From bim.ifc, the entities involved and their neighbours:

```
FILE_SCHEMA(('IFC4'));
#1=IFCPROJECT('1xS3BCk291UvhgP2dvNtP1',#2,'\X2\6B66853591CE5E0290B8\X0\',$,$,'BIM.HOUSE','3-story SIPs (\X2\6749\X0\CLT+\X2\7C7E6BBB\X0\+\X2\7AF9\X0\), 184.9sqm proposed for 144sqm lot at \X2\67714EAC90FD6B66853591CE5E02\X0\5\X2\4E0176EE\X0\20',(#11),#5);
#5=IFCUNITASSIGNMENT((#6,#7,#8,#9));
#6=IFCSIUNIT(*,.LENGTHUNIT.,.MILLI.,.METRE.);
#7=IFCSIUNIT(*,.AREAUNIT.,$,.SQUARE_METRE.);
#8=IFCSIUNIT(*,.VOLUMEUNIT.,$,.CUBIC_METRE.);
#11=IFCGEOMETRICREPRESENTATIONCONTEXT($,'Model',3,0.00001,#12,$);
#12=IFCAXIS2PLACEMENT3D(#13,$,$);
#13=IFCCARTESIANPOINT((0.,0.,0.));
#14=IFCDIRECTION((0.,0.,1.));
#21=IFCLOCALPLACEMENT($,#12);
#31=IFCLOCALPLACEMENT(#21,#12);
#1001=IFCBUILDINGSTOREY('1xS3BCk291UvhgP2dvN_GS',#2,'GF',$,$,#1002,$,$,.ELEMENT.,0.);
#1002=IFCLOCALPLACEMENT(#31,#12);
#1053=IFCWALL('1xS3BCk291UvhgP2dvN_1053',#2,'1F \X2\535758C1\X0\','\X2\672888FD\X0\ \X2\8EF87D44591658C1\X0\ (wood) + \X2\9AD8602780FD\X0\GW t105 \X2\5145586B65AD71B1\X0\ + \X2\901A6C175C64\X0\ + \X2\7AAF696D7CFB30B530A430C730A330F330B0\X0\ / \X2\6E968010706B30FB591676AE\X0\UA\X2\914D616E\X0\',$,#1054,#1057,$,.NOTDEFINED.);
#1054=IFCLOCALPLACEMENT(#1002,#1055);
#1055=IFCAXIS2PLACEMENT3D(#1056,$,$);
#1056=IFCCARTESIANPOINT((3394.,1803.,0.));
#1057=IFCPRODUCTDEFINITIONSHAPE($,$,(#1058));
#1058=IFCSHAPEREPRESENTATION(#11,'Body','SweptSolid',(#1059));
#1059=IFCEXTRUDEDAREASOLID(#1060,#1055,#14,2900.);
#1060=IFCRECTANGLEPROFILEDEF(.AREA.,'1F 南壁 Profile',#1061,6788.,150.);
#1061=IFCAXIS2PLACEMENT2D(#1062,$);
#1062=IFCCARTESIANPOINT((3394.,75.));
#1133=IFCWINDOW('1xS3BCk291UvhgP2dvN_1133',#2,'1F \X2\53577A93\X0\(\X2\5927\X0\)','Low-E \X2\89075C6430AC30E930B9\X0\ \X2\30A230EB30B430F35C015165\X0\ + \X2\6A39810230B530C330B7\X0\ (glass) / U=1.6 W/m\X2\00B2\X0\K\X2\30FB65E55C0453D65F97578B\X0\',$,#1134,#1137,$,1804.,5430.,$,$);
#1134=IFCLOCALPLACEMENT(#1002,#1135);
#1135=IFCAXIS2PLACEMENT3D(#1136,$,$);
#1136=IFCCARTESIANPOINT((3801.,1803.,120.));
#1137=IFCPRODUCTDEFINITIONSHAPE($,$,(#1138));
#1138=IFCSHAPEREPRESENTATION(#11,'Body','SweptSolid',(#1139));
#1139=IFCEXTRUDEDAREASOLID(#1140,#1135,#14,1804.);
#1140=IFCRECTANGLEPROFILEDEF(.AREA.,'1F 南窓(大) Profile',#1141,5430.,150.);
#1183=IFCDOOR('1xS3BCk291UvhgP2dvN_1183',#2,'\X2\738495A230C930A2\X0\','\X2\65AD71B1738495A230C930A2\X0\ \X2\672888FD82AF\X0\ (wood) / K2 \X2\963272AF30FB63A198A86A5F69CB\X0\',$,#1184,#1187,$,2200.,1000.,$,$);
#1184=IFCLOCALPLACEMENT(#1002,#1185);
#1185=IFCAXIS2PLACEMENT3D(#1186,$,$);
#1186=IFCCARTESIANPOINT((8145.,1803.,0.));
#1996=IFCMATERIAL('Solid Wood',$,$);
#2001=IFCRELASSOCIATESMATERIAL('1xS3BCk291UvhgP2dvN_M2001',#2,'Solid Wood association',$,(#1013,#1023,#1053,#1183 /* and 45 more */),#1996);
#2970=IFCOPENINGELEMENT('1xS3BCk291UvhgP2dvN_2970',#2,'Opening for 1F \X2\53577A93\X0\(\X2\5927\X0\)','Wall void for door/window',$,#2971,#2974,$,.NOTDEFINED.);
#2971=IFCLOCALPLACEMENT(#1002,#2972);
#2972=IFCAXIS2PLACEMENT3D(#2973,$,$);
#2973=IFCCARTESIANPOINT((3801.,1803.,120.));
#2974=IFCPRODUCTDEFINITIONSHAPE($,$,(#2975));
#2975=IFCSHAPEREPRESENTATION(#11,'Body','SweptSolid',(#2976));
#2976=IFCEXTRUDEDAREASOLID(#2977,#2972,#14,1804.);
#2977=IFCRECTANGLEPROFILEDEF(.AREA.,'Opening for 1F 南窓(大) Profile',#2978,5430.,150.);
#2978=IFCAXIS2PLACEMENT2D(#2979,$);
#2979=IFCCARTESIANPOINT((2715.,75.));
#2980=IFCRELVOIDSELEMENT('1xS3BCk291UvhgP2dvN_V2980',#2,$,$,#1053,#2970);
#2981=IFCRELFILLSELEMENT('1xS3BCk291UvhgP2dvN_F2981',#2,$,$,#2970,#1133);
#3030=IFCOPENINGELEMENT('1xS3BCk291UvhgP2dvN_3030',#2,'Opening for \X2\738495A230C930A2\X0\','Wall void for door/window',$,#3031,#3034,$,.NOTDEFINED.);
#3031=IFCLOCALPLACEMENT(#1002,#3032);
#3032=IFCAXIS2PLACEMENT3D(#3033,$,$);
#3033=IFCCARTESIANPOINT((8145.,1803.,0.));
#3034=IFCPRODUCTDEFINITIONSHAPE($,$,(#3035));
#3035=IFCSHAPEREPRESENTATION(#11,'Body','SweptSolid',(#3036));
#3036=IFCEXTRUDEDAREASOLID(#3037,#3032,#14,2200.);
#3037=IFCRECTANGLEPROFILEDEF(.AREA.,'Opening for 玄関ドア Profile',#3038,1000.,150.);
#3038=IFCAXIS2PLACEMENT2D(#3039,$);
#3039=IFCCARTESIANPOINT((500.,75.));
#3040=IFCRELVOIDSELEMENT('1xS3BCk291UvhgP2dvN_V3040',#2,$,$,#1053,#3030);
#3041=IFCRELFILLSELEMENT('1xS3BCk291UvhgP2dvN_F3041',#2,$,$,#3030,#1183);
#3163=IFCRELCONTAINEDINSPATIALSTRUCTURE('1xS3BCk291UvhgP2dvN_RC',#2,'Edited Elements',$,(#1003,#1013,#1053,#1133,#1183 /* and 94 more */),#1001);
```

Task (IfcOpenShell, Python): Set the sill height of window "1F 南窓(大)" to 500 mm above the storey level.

```python
import numpy as np
import ifcopenshell
import ifcopenshell.api.geometry
import ifcopenshell.geom
import ifcopenshell.util.element
import ifcopenshell.util.placement
import ifcopenshell.util.shape
import ifcopenshell.util.unit

model = ifcopenshell.open("bim.ifc")
unit_scale = ifcopenshell.util.unit.calculate_unit_scale(model)

window = model.by_guid("1xS3BCk291UvhgP2dvN_1133")
opening = window.FillsVoids[0].RelatingOpeningElement
storey = ifcopenshell.util.element.get_container(window, ifc_class="IfcBuildingStorey")
level = ifcopenshell.util.placement.get_local_placement(storey.ObjectPlacement)[2, 3]

# The opening's origin need not be at the sill, so measure its lowest point.
shape = ifcopenshell.geom.create_shape(ifcopenshell.geom.settings(), opening)
bottom = ifcopenshell.util.shape.get_shape_bottom_elevation(shape, shape.geometry) / unit_scale
dz = level + 500.0 - bottom

shift = np.array([0.0, 0.0, dz])
# The window is not placed relative to its opening, so move both.
for product in (opening, window):
    matrix = ifcopenshell.util.placement.get_local_placement(product.ObjectPlacement)
    matrix[:3, 3] += shift
    ifcopenshell.api.geometry.edit_object_placement(model, product=product, matrix=matrix, is_si=False)

print(f"moved by {dz * unit_scale:+.3f} m")

model.write("bim_updated.ifc")
```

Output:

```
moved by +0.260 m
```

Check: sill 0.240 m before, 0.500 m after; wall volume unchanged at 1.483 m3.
